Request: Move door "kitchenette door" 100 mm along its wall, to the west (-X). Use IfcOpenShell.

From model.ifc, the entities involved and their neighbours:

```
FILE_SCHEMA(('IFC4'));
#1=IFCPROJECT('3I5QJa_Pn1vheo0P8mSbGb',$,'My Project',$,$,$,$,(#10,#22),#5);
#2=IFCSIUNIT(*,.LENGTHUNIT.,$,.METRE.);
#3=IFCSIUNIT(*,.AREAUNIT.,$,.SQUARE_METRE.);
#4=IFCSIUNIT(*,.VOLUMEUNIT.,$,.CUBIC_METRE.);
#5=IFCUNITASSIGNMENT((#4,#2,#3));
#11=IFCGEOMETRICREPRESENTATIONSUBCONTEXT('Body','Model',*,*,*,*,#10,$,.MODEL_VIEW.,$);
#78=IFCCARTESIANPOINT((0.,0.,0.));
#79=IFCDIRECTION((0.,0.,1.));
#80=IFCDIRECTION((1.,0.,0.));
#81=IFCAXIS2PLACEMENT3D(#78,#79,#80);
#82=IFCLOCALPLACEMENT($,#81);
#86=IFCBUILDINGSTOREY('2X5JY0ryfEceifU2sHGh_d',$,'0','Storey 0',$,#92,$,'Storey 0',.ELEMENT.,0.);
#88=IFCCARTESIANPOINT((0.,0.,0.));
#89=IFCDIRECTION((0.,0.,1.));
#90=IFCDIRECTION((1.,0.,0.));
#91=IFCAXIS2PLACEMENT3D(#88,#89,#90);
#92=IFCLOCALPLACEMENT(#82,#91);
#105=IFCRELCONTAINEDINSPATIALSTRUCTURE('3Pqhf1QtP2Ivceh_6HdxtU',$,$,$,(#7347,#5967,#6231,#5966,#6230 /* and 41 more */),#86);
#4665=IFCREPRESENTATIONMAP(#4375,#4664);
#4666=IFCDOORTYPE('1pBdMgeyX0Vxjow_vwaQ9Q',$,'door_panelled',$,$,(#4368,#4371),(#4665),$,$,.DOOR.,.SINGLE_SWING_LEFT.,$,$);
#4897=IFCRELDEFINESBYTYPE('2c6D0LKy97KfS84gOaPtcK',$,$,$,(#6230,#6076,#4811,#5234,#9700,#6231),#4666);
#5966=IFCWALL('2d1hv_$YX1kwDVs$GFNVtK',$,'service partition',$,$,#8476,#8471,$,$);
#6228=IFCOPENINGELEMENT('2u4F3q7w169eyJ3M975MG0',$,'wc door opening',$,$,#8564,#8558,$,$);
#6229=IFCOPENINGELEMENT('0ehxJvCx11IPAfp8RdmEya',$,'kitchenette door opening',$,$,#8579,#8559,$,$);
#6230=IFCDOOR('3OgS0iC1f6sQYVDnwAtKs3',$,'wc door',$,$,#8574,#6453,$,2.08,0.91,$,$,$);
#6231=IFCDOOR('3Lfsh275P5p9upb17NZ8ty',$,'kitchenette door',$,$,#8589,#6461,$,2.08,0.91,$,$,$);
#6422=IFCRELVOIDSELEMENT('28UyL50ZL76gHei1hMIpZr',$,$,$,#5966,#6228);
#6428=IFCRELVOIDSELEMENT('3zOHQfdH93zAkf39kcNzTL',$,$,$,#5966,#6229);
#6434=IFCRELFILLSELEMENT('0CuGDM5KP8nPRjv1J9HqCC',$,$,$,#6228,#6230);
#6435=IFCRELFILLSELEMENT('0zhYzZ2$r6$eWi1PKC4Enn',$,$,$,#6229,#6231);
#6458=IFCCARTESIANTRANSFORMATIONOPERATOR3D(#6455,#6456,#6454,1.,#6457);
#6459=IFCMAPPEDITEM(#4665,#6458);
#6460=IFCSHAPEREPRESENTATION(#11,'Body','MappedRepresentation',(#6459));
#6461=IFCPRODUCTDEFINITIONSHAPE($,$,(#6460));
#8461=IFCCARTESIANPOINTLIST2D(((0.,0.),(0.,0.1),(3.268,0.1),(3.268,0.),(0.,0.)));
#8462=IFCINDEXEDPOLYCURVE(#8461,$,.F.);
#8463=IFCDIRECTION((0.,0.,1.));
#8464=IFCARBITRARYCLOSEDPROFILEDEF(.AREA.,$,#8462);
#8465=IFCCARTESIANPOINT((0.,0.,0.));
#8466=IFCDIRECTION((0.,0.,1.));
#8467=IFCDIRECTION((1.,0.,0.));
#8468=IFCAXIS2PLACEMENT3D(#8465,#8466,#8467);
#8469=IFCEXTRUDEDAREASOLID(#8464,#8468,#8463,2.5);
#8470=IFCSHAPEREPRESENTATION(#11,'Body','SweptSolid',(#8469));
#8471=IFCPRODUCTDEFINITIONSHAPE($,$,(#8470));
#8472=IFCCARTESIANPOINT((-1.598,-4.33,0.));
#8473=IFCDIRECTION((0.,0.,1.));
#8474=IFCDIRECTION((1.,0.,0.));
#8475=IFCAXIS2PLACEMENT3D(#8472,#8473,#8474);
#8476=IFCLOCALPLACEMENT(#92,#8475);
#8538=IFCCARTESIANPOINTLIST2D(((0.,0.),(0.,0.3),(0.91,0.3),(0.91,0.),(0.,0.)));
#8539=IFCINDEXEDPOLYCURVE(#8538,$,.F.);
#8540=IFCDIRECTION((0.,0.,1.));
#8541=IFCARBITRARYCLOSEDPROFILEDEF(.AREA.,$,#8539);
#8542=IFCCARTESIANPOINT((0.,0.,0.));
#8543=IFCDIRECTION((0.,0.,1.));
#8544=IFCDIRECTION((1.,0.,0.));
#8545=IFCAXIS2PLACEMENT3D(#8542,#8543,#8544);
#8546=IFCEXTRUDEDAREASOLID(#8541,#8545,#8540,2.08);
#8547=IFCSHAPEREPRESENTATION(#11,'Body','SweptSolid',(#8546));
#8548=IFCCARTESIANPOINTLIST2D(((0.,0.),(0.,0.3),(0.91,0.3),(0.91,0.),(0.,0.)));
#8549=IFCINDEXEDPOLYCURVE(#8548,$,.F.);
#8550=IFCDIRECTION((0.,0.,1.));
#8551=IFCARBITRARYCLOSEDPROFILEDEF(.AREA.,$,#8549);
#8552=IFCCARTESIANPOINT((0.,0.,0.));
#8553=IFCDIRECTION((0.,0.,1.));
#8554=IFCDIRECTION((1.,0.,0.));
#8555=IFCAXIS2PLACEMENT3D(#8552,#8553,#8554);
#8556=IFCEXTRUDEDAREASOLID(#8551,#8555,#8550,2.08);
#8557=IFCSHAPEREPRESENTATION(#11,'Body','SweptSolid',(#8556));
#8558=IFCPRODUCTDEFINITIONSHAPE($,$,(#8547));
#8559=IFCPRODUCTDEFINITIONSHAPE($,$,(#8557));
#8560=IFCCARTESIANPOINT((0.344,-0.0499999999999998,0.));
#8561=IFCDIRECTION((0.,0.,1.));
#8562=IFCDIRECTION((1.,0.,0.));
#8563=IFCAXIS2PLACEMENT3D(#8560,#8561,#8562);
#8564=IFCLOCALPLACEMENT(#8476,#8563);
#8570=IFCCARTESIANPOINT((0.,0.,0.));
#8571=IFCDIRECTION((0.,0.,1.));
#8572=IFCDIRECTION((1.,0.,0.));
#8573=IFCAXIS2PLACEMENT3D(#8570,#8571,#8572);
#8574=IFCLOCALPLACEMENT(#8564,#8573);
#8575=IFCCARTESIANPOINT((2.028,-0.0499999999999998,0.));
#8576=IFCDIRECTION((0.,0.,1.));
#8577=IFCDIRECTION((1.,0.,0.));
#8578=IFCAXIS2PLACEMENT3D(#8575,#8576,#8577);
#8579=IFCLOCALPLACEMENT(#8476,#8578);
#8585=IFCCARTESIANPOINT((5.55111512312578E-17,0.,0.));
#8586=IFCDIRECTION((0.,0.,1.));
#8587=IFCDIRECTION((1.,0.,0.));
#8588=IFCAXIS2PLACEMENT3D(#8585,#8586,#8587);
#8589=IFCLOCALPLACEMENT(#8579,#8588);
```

```python
import ifcopenshell
import ifcopenshell.api.geometry
import ifcopenshell.util.placement
import ifcopenshell.util.unit

model = ifcopenshell.open("model.ifc")
unit_scale = ifcopenshell.util.unit.calculate_unit_scale(model)

door = model.by_guid("3Lfsh275P5p9upb17NZ8ty")
opening = door.FillsVoids[0].RelatingOpeningElement
wall = opening.VoidsElements[0].RelatingBuildingElement

wall_matrix = ifcopenshell.util.placement.get_local_placement(wall.ObjectPlacement)
shift = wall_matrix[:3, 0] * -0.1 / unit_scale
before = ifcopenshell.util.placement.get_local_placement(door.ObjectPlacement)[:3, 3].copy()

# The door is placed relative to its opening, so it follows when the opening moves.
matrix = ifcopenshell.util.placement.get_local_placement(opening.ObjectPlacement)
matrix[:3, 3] += shift
ifcopenshell.api.geometry.edit_object_placement(
    model, product=opening, matrix=matrix, is_si=False, should_transform_children=True
)

after = ifcopenshell.util.placement.get_local_placement(door.ObjectPlacement)[:3, 3]
print("door moved by", (after - before).round(3) + 0.0)

model.write("model_updated.ifc")
```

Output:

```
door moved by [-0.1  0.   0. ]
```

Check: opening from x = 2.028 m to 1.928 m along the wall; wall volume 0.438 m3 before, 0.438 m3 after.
